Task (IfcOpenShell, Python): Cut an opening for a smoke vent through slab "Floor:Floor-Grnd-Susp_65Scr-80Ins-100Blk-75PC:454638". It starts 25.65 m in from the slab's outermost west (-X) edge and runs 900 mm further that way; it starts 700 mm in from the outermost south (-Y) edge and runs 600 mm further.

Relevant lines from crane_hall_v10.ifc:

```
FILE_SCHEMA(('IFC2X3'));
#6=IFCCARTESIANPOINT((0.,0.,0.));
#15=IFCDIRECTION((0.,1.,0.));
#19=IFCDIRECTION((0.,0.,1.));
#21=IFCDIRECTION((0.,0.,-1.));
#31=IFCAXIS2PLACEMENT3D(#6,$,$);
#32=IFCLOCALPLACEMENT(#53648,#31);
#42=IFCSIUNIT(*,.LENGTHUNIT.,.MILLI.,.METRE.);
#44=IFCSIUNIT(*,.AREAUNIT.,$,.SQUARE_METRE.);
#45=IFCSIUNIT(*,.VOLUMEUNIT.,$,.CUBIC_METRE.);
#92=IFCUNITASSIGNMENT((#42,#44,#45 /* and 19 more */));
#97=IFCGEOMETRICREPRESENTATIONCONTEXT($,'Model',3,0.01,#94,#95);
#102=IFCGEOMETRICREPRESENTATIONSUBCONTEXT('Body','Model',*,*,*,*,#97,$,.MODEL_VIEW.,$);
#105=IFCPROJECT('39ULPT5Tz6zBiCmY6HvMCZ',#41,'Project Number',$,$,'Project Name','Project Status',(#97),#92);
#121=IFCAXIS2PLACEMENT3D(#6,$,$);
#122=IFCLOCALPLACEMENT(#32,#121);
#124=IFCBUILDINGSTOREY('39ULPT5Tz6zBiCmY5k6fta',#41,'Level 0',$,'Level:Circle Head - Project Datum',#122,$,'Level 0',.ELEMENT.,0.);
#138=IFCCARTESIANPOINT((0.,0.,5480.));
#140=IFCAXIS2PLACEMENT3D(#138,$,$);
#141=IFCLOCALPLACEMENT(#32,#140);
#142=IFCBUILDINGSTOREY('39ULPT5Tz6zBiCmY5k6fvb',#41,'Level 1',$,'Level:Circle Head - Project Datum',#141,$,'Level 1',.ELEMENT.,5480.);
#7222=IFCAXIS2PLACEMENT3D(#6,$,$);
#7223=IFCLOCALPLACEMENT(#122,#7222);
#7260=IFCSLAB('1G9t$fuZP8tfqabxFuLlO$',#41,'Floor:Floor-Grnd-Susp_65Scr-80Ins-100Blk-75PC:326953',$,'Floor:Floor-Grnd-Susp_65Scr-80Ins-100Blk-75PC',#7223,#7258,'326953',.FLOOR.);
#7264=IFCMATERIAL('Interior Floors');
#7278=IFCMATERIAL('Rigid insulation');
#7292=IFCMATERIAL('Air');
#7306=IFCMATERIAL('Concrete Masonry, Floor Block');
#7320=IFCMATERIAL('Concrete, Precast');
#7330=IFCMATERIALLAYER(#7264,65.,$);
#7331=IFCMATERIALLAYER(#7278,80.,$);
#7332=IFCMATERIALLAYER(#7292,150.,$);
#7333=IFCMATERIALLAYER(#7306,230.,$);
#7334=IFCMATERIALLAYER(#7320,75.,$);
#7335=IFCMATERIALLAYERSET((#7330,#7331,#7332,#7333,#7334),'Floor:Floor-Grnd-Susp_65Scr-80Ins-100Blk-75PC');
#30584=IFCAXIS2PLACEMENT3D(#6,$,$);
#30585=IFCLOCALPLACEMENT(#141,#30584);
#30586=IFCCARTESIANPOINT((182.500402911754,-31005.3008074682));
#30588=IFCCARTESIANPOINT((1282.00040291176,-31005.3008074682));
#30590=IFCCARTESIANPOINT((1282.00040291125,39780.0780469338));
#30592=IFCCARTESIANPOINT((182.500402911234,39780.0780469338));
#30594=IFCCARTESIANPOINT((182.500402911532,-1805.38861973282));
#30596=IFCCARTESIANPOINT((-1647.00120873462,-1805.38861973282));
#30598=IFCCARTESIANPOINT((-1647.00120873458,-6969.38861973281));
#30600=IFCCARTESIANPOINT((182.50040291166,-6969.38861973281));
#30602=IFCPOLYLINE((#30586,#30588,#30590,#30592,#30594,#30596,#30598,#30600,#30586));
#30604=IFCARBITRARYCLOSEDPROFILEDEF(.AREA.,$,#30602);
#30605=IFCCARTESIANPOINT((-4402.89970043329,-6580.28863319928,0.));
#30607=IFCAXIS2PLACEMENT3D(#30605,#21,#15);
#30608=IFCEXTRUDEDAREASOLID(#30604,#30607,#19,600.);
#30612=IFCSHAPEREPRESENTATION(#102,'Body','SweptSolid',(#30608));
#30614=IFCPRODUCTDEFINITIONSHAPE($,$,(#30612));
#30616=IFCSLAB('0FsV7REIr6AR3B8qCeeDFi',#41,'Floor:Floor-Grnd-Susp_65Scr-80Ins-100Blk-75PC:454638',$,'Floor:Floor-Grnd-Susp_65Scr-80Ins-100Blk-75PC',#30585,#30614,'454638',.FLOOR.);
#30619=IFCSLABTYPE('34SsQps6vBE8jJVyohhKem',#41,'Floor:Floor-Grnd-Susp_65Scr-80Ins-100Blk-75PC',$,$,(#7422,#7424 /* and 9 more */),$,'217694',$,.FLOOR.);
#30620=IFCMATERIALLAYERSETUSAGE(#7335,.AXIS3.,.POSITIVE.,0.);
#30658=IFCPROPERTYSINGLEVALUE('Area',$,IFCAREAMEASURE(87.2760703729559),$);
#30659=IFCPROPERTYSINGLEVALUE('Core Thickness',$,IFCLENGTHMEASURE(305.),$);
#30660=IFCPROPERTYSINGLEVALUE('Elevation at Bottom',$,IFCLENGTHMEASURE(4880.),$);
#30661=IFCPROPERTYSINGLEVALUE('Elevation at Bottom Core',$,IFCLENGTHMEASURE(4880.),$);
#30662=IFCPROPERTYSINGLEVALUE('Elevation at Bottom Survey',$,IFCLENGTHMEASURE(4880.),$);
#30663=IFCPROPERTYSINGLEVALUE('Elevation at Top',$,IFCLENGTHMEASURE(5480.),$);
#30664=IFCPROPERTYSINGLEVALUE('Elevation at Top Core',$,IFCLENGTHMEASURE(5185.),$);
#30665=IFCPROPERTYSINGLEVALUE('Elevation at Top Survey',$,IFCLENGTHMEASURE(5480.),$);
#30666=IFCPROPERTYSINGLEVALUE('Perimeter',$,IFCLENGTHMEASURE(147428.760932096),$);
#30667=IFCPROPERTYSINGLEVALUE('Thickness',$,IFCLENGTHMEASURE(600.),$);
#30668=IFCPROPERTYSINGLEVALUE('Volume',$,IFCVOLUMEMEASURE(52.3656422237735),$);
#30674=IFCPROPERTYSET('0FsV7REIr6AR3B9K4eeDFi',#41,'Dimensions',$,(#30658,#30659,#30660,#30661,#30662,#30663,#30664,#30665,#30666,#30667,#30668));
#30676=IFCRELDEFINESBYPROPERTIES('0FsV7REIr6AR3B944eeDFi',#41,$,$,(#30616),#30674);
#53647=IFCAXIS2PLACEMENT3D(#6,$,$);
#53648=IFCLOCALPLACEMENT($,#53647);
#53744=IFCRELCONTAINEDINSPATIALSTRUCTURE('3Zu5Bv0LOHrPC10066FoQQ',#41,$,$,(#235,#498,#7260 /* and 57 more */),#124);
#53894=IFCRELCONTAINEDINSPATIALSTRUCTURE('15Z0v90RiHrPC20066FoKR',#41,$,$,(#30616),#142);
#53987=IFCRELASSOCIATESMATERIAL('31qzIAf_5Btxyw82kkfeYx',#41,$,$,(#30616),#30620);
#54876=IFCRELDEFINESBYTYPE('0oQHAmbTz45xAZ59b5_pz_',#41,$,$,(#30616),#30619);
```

```python
import numpy as np
import ifcopenshell
import ifcopenshell.api.feature
import ifcopenshell.api.geometry
import ifcopenshell.api.pset
import ifcopenshell.api.root
import ifcopenshell.geom
import ifcopenshell.util.element
import ifcopenshell.util.placement
import ifcopenshell.util.representation
import ifcopenshell.util.shape
import ifcopenshell.util.unit

model = ifcopenshell.open("crane_hall_v10.ifc")
unit_scale = ifcopenshell.util.unit.calculate_unit_scale(model)
area_scale = ifcopenshell.util.unit.calculate_unit_scale(model, "AREAUNIT")
volume_scale = ifcopenshell.util.unit.calculate_unit_scale(model, "VOLUMEUNIT")
settings = ifcopenshell.geom.settings()


def volume(element):
    """Net volume in cubic metres, openings subtracted."""
    shape = ifcopenshell.geom.create_shape(settings, element)
    return ifcopenshell.util.shape.get_volume(shape.geometry)


slab = model.by_guid("0FsV7REIr6AR3B8qCeeDFi")
before = volume(slab)

# Extent in the slab's own axes, in metres. The edges named are its -X and -Y sides.
slab_shape = ifcopenshell.geom.create_shape(settings, slab)
vertices = ifcopenshell.util.shape.get_vertices(slab_shape.geometry)
x_min, y_min, bottom = vertices.min(axis=0)
top = vertices[:, 2].max()

opening = ifcopenshell.api.root.create_entity(model, ifc_class="IfcOpeningElement", name="Smoke vent opening")
context = ifcopenshell.util.representation.get_context(model, "Model", "Body", "MODEL_VIEW")
width, depth = 0.9, 0.6
outline = [(0.0, 0.0), (width, 0.0), (width, depth), (0.0, depth), (0.0, 0.0)]
# Overshoot both faces by 50 mm so the cut is clean.
shape = ifcopenshell.api.geometry.add_slab_representation(
    model, context=context, depth=top - bottom + 0.1, polyline=outline
)
ifcopenshell.api.geometry.assign_representation(model, product=opening, representation=shape)

matrix = ifcopenshell.util.placement.get_local_placement(slab.ObjectPlacement)
matrix[:, 3] = matrix @ np.append(np.array([x_min + 25.65, y_min + 0.7, bottom - 0.05]) / unit_scale, 1.0)
ifcopenshell.api.geometry.edit_object_placement(model, product=opening, matrix=matrix, is_si=False)
ifcopenshell.api.feature.add_feature(model, feature=opening, element=slab)

after = volume(slab)

# Update the slab's stored quantities.
pset = model.by_id(ifcopenshell.util.element.get_pset(slab, "Dimensions", should_inherit=False)["id"])
ifcopenshell.api.pset.edit_pset(model, pset=pset, properties={
    "Area": model.create_entity("IfcAreaMeasure", after / (top - bottom) / area_scale),
    "Volume": model.create_entity("IfcVolumeMeasure", after / volume_scale),
})

print(f"slab volume {before:.3f} -> {after:.3f} m3")

model.write("crane_hall_v10_v2.ifc")
```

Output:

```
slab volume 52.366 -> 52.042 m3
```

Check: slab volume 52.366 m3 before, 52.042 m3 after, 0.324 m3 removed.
